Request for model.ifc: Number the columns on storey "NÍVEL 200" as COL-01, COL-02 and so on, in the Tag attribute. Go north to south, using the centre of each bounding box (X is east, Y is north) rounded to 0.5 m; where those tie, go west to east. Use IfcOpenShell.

First a look at what the model holds.

```python
import ifcopenshell
import ifcopenshell.util.element
import ifcopenshell.util.placement

model = ifcopenshell.open("model.ifc")
print(model.schema)
storey = next(s for s in model.by_type("IfcBuildingStorey") if s.Name == "NÍVEL 200")
columns = [e for e in ifcopenshell.util.element.get_decomposition(storey) if e.is_a("IfcColumn")]
for e in sorted(columns, key=lambda e: e.id()):
    origin = ifcopenshell.util.placement.get_local_placement(e.ObjectPlacement)[:3, 3]
    print(e.id(), e.Tag, e.Name, origin.round(2) + 0.0, sep=" | ")
```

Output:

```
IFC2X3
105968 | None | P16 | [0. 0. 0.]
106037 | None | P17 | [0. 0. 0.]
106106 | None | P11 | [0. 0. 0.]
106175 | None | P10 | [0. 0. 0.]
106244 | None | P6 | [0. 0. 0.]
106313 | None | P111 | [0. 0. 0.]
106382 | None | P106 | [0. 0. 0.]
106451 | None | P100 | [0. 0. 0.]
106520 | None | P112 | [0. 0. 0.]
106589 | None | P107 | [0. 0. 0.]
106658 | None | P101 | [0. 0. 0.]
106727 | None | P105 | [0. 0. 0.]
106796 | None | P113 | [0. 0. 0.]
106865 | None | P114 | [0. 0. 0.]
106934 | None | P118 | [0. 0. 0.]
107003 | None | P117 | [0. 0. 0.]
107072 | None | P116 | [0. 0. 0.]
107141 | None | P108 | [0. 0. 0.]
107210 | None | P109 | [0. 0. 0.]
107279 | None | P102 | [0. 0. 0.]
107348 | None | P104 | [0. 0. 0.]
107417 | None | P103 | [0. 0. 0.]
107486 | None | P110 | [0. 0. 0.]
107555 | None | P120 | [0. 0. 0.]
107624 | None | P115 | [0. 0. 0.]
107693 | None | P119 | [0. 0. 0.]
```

```python
import ifcopenshell
import ifcopenshell.geom
import ifcopenshell.util.element
import ifcopenshell.util.shape

model = ifcopenshell.open("model.ifc")
settings = ifcopenshell.geom.settings()
settings.set("use-world-coords", True)


def centre(element):
    shape = ifcopenshell.geom.create_shape(settings, element)
    return ifcopenshell.util.shape.get_bbox_centroid(shape.geometry)


storey = next(s for s in model.by_type("IfcBuildingStorey") if s.Name == "NÍVEL 200")
columns = [e for e in ifcopenshell.util.element.get_decomposition(storey) if e.is_a("IfcColumn")]

# Insertion points can sit at a corner or the storey origin, so sort by the geometry (in metres).
centres = {e: centre(e) for e in columns}
columns.sort(key=lambda e: (-round(centres[e][1] / 0.5), centres[e][0]))

for i, e in enumerate(columns, start=1):
    number = f"COL-{i:02d}"
    e.Tag = number
    print(e.id(), number)

model.write("model_v2.ifc")
```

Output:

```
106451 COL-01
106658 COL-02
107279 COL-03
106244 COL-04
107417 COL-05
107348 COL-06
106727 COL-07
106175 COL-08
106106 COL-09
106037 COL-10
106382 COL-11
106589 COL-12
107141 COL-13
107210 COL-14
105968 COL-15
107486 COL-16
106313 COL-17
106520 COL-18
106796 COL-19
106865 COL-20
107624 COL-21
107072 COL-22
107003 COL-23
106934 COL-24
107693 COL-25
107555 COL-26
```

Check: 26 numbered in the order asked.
